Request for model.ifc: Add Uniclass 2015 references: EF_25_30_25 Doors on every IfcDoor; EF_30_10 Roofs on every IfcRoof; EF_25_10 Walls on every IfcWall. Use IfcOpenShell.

First a look at what the model holds.

```python
import ifcopenshell

model = ifcopenshell.open("model.ifc")
print(model.schema)
print("classifications:", [c.Name for c in model.by_type("IfcClassification")])
for ifc_class in ("IfcDoor", "IfcRoof", "IfcStair", "IfcWall", "IfcWindow"):
    print(ifc_class, len(model.by_type(ifc_class)))
```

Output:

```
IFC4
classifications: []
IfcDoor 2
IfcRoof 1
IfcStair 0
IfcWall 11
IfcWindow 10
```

```python
import ifcopenshell
import ifcopenshell.api.classification

model = ifcopenshell.open("model.ifc")

system = ifcopenshell.api.classification.add_classification(model, classification="Uniclass 2015")

codes = {
    "IfcDoor": ("EF_25_30_25", "Doors"),
    "IfcRoof": ("EF_30_10", "Roofs"),
    "IfcWall": ("EF_25_10", "Walls"),
}
for ifc_class, (code, name) in codes.items():
    products = model.by_type(ifc_class)
    ifcopenshell.api.classification.add_reference(
        model, products=products, classification=system, identification=code, name=name
    )
    print(code, len(products))

model.write("model_v2.ifc")
```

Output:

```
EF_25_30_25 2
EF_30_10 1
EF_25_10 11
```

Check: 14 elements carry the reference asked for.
